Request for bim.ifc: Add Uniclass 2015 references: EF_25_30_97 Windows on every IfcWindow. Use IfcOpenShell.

First a look at what the model holds.

```python
import ifcopenshell

model = ifcopenshell.open("bim.ifc")
print(model.schema)
print("classifications:", [c.Name for c in model.by_type("IfcClassification")])
for ifc_class in ("IfcDoor", "IfcRoof", "IfcStair", "IfcWall", "IfcWindow"):
    print(ifc_class, len(model.by_type(ifc_class)))
```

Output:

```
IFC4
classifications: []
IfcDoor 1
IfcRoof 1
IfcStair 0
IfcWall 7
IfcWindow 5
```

```python
import ifcopenshell
import ifcopenshell.api.classification

model = ifcopenshell.open("bim.ifc")

system = ifcopenshell.api.classification.add_classification(model, classification="Uniclass 2015")

codes = {
    "IfcWindow": ("EF_25_30_97", "Windows"),
}
for ifc_class, (code, name) in codes.items():
    products = model.by_type(ifc_class)
    ifcopenshell.api.classification.add_reference(
        model, products=products, classification=system, identification=code, name=name
    )
    print(code, len(products))

model.write("bim-out.ifc")
```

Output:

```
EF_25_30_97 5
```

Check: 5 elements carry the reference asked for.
